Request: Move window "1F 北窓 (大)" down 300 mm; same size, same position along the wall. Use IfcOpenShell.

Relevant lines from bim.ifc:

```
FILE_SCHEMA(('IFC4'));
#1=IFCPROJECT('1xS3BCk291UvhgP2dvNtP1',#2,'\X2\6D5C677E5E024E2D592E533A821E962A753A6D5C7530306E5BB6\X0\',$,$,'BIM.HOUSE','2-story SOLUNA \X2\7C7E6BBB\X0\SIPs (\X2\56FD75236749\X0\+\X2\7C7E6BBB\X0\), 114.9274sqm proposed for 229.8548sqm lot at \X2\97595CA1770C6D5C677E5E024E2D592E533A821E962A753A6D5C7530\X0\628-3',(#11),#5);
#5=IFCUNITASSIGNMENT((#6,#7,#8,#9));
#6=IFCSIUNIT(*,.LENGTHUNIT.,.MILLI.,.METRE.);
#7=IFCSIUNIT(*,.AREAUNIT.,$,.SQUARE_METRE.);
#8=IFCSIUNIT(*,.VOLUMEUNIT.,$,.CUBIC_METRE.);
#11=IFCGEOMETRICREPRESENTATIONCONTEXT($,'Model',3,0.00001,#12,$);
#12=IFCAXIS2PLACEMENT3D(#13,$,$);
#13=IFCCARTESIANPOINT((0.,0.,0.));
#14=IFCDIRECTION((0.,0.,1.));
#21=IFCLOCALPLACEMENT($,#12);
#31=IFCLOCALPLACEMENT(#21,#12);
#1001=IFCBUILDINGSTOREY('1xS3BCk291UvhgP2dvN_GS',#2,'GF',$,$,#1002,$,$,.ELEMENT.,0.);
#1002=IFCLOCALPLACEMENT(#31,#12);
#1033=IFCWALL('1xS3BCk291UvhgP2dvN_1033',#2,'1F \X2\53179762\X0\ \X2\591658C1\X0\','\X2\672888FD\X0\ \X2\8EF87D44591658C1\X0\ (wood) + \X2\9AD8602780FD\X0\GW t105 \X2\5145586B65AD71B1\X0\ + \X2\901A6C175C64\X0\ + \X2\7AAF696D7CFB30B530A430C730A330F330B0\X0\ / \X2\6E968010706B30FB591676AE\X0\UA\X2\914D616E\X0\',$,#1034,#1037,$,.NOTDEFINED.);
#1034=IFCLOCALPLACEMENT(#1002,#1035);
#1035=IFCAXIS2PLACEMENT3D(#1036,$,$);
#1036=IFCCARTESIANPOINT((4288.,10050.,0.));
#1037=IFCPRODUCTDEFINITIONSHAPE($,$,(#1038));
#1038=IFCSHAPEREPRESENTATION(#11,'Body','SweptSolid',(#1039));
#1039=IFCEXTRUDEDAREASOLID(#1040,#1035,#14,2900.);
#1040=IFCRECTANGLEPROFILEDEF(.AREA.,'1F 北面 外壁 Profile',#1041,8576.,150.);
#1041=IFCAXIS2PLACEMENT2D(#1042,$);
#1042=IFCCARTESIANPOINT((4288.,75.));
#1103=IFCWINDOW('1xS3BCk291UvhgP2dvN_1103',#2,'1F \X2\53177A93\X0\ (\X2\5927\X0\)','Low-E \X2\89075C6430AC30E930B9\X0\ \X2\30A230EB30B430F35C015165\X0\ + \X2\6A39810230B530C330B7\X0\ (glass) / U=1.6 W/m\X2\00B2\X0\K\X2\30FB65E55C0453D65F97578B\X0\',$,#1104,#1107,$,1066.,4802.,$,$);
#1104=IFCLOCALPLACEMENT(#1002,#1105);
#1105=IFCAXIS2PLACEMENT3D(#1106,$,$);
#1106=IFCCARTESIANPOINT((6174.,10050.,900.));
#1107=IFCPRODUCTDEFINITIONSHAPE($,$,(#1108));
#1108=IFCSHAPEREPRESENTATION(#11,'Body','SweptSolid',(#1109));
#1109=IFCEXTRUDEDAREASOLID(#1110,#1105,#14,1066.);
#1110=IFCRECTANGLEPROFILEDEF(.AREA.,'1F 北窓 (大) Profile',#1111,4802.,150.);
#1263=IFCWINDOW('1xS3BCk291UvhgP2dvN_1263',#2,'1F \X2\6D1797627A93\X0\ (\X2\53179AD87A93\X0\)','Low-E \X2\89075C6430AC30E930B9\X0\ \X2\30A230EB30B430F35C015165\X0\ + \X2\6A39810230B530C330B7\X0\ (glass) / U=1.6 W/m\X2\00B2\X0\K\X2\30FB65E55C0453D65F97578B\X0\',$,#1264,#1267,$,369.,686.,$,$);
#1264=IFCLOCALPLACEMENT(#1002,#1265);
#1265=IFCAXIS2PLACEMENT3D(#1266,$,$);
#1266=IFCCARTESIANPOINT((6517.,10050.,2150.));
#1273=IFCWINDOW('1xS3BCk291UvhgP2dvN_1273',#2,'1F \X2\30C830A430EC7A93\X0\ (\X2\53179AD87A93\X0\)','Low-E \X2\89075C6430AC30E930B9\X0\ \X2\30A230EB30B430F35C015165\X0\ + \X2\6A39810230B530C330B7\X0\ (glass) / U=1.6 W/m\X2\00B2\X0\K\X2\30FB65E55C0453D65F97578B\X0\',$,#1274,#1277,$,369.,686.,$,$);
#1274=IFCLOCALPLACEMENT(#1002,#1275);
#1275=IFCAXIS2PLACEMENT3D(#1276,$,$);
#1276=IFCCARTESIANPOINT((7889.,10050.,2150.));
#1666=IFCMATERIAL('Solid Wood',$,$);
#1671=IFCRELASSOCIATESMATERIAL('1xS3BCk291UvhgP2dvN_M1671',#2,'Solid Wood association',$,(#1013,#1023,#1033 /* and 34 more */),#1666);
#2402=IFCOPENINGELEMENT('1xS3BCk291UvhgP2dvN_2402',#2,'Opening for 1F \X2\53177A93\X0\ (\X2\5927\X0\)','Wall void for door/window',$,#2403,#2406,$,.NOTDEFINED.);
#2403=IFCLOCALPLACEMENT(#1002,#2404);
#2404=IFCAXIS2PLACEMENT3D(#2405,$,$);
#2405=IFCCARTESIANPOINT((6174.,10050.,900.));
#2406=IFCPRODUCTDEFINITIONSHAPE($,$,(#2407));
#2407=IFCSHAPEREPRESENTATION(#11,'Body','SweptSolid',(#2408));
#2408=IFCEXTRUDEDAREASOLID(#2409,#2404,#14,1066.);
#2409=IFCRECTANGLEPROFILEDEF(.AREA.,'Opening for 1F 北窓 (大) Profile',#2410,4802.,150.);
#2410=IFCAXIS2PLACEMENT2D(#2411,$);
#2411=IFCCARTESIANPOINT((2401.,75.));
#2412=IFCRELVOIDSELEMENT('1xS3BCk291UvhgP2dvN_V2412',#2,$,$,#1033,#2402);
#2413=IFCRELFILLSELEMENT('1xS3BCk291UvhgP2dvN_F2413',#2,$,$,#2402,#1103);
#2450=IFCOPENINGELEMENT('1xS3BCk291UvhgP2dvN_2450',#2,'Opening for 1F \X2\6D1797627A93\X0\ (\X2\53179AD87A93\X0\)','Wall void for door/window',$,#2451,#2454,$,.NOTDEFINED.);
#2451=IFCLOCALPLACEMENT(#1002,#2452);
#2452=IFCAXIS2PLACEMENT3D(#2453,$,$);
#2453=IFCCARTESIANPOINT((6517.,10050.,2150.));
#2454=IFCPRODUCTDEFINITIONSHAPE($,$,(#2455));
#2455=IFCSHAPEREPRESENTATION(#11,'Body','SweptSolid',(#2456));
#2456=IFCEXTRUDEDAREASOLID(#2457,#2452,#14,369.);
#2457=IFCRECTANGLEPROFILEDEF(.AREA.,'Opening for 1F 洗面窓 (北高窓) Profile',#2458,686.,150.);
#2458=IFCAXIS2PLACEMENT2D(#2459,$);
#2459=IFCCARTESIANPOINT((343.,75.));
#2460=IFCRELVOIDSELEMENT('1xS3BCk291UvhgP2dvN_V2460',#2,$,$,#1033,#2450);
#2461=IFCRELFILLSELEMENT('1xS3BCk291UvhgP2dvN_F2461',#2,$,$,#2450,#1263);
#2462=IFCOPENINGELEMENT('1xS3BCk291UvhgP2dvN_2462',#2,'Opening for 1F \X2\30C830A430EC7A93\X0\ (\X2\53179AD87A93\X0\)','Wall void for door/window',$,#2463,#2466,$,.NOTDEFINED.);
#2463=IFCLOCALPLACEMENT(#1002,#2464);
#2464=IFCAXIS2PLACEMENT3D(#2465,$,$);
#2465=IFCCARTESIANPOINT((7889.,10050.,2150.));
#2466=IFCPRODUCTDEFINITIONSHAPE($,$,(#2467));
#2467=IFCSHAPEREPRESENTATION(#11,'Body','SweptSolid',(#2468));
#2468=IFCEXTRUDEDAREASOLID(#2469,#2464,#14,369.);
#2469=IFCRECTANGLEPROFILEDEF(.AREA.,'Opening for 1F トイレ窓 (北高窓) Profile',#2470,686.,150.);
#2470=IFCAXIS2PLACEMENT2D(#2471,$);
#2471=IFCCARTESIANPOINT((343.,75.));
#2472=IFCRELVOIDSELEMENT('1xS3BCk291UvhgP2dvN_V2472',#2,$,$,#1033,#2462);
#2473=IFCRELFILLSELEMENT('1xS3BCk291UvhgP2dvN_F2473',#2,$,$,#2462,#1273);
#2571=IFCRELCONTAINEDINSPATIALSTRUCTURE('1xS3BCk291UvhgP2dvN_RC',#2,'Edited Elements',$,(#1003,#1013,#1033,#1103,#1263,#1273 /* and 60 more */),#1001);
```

```python
import numpy as np
import ifcopenshell
import ifcopenshell.api.geometry
import ifcopenshell.util.placement
import ifcopenshell.util.unit

model = ifcopenshell.open("bim.ifc")
unit_scale = ifcopenshell.util.unit.calculate_unit_scale(model)

window = model.by_guid("1xS3BCk291UvhgP2dvN_1103")
opening = window.FillsVoids[0].RelatingOpeningElement
dz = -0.3 / unit_scale

shift = np.array([0.0, 0.0, dz])
# The window is not placed relative to its opening, so move both.
for product in (opening, window):
    matrix = ifcopenshell.util.placement.get_local_placement(product.ObjectPlacement)
    matrix[:3, 3] += shift
    ifcopenshell.api.geometry.edit_object_placement(model, product=product, matrix=matrix, is_si=False)

print(f"moved by {dz * unit_scale:+.3f} m")

model.write("bim_edited.ifc")
```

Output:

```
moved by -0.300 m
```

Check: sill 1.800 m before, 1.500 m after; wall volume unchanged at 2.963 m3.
